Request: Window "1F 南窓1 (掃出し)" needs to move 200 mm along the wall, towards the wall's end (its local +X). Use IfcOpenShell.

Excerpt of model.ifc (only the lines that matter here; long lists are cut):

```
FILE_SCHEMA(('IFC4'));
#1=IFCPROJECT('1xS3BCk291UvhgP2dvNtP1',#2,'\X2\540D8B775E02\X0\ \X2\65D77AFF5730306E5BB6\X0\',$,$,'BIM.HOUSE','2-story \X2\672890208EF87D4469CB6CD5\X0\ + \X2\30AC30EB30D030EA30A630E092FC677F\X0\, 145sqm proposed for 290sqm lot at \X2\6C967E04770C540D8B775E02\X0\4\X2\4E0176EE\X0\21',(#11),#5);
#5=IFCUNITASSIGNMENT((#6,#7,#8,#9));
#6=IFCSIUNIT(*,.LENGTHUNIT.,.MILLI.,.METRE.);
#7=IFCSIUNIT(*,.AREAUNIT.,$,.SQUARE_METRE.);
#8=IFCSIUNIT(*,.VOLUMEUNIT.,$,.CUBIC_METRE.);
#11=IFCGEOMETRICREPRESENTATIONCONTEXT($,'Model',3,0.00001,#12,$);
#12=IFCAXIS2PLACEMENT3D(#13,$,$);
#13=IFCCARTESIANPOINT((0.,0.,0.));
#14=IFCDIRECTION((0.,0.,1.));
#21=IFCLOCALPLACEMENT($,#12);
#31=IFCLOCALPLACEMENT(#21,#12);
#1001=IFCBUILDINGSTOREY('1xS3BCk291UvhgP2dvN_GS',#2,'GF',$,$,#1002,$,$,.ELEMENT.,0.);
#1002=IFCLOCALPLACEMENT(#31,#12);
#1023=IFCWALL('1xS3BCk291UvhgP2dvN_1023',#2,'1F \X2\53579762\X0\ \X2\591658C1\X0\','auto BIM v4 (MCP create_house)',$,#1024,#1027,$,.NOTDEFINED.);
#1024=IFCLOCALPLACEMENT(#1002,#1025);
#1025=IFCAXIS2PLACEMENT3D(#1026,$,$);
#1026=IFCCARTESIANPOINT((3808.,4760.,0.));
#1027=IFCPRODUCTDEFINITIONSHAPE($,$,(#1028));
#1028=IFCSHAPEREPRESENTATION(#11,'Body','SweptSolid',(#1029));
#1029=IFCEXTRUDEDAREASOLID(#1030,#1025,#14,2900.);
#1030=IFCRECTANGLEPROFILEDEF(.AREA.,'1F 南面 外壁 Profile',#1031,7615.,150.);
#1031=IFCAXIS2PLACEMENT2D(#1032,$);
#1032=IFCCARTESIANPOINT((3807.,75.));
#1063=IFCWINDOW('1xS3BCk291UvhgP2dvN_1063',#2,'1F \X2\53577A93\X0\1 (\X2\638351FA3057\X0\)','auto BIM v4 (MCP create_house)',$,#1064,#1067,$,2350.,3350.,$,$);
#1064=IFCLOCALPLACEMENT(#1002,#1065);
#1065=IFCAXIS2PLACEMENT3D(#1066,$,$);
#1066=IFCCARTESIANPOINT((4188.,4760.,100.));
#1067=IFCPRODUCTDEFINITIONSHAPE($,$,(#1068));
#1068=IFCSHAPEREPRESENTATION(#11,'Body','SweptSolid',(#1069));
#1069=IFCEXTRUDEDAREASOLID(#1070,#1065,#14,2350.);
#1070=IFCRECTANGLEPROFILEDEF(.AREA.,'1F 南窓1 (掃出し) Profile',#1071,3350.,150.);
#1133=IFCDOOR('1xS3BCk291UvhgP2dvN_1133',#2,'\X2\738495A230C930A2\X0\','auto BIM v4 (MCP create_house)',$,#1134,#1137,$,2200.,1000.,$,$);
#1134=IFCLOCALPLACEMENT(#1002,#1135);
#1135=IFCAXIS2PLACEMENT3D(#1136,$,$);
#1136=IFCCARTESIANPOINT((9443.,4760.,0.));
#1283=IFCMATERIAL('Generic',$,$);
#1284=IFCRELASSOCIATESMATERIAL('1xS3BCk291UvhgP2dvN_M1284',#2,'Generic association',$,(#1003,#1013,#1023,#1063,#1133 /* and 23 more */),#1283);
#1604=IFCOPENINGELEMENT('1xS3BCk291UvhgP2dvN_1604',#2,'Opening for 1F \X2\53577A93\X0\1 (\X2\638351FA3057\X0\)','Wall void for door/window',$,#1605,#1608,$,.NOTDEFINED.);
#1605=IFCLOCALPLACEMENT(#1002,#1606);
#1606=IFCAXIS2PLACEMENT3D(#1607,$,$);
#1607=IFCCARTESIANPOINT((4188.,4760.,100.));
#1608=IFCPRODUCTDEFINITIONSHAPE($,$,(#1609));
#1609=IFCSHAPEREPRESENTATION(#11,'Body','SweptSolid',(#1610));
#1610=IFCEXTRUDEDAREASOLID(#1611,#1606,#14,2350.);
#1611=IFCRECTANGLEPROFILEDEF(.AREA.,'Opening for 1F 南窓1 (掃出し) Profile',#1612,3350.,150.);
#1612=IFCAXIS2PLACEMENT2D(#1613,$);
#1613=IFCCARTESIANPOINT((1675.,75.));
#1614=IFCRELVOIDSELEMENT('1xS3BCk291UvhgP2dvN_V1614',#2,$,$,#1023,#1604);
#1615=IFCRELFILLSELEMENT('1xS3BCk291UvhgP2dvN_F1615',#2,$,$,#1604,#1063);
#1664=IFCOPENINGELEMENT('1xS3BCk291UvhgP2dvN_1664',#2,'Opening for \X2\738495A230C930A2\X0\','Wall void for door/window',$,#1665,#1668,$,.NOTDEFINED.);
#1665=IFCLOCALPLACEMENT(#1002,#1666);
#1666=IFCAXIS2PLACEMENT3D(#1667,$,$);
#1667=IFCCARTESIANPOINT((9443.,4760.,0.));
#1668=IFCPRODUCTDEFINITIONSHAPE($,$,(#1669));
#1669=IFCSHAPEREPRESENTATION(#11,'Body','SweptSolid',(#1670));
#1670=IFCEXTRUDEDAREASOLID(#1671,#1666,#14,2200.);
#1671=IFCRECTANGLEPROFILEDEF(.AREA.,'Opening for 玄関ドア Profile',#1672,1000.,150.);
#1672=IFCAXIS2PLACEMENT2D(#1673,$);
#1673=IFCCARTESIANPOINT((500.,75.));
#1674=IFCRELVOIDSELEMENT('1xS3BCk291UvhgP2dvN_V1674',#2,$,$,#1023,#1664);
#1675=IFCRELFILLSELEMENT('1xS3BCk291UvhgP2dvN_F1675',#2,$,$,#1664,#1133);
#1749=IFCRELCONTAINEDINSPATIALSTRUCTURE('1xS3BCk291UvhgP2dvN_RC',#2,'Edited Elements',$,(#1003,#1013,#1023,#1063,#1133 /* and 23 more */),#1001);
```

```python
import ifcopenshell
import ifcopenshell.api.geometry
import ifcopenshell.util.placement

model = ifcopenshell.open("model.ifc")

window = model.by_guid("1xS3BCk291UvhgP2dvN_1063")
opening = window.FillsVoids[0].RelatingOpeningElement
wall = opening.VoidsElements[0].RelatingBuildingElement

wall_matrix = ifcopenshell.util.placement.get_local_placement(wall.ObjectPlacement)
shift = wall_matrix[:3, 0] * 200.0
before = ifcopenshell.util.placement.get_local_placement(window.ObjectPlacement)[:3, 3].copy()

# The window is not placed relative to its opening, so move both.
for product in (opening, window):
    matrix = ifcopenshell.util.placement.get_local_placement(product.ObjectPlacement)
    matrix[:3, 3] += shift
    ifcopenshell.api.geometry.edit_object_placement(model, product=product, matrix=matrix, is_si=False)

after = ifcopenshell.util.placement.get_local_placement(window.ObjectPlacement)[:3, 3]
print("window moved by", (after - before).round(3) + 0.0)

model.write("model_edited.ifc")
```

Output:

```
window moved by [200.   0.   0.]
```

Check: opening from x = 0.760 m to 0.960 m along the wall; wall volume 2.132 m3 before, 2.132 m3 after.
